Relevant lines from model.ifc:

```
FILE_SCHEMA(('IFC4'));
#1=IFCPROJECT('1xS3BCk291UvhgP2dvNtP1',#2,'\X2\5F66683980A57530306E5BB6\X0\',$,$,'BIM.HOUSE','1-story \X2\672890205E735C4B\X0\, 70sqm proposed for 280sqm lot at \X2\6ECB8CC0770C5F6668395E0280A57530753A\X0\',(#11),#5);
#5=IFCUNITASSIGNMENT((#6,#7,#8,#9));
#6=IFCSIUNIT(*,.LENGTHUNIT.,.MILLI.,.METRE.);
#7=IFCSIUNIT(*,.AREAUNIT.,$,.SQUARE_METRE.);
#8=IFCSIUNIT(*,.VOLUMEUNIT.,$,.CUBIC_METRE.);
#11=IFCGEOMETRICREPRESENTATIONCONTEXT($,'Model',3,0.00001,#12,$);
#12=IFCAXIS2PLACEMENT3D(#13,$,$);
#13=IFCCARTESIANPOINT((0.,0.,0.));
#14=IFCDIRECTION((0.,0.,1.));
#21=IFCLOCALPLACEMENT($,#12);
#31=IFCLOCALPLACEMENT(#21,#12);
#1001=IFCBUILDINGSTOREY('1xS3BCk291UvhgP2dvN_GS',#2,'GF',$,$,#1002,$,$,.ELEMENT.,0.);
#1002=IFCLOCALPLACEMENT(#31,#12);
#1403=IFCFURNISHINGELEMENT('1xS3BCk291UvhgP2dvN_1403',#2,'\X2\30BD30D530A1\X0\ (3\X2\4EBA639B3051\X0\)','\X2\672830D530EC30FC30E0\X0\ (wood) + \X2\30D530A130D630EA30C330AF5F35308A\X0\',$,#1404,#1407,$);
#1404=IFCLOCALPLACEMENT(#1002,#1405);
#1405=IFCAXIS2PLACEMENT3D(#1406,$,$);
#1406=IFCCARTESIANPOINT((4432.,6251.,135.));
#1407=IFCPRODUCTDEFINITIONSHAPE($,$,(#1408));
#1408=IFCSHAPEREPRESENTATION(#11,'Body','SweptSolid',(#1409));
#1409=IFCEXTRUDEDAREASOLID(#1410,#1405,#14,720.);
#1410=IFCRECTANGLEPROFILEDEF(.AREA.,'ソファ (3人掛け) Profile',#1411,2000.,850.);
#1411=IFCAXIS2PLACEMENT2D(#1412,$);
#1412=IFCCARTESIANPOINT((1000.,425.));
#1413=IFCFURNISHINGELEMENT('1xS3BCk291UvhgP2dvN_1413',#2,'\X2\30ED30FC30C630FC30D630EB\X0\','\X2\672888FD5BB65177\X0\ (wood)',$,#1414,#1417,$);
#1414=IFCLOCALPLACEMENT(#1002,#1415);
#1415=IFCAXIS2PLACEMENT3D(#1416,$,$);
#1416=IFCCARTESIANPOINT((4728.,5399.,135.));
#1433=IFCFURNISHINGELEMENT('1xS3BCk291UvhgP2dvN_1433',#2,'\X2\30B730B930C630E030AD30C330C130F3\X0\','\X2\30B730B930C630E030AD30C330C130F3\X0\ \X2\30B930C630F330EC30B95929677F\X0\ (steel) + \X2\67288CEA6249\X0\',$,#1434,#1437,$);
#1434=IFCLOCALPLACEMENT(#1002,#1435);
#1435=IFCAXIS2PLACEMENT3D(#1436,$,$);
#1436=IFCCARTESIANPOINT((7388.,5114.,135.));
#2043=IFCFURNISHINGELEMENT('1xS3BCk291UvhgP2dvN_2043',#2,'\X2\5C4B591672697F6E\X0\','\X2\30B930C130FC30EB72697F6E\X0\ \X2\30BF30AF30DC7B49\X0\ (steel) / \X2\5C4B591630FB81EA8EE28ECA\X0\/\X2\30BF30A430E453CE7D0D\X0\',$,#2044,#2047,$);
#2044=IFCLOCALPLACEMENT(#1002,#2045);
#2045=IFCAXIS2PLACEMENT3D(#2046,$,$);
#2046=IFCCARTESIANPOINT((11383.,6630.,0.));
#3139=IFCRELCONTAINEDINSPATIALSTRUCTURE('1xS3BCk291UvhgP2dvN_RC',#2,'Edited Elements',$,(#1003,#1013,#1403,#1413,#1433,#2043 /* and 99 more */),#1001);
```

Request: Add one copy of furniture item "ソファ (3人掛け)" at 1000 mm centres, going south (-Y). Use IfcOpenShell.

```python
import numpy as np
import ifcopenshell
import ifcopenshell.api.geometry
import ifcopenshell.api.root
import ifcopenshell.util.element
import ifcopenshell.util.placement
import ifcopenshell.util.unit

model = ifcopenshell.open("model.ifc")
unit_scale = ifcopenshell.util.unit.calculate_unit_scale(model)


def reuse_history(source, copy):
    """copy_class also copies each property set's owner history, people and application; keep the originals."""
    for rel in copy.IsDefinedBy:
        if rel.is_a("IfcRelDefinesByProperties") and (history := rel.RelatingPropertyDefinition.OwnerHistory):
            rel.RelatingPropertyDefinition.OwnerHistory = source.OwnerHistory
            ifcopenshell.util.element.remove_deep2(model, history)


source = model.by_guid("1xS3BCk291UvhgP2dvN_1403")
base = ifcopenshell.util.placement.get_local_placement(source.ObjectPlacement)
step = np.array([0.0, -1.0, 0.0]) * 1 / unit_scale

for i in range(1, 2):
    copy = ifcopenshell.api.root.copy_class(model, product=source)
    copy.Representation = ifcopenshell.util.element.copy_deep(
        model, source.Representation, exclude=["IfcGeometricRepresentationContext", "IfcRepresentationMap"]
    )
    reuse_history(source, copy)
    matrix = base.copy()
    matrix[:3, 3] += i * step
    print("added at", matrix[:3, 3].round(3) + 0.0)
    ifcopenshell.api.geometry.edit_object_placement(model, product=copy, matrix=matrix, is_si=False)

model.write("model_rev.ifc")
```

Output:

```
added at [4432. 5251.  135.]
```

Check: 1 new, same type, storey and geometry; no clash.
